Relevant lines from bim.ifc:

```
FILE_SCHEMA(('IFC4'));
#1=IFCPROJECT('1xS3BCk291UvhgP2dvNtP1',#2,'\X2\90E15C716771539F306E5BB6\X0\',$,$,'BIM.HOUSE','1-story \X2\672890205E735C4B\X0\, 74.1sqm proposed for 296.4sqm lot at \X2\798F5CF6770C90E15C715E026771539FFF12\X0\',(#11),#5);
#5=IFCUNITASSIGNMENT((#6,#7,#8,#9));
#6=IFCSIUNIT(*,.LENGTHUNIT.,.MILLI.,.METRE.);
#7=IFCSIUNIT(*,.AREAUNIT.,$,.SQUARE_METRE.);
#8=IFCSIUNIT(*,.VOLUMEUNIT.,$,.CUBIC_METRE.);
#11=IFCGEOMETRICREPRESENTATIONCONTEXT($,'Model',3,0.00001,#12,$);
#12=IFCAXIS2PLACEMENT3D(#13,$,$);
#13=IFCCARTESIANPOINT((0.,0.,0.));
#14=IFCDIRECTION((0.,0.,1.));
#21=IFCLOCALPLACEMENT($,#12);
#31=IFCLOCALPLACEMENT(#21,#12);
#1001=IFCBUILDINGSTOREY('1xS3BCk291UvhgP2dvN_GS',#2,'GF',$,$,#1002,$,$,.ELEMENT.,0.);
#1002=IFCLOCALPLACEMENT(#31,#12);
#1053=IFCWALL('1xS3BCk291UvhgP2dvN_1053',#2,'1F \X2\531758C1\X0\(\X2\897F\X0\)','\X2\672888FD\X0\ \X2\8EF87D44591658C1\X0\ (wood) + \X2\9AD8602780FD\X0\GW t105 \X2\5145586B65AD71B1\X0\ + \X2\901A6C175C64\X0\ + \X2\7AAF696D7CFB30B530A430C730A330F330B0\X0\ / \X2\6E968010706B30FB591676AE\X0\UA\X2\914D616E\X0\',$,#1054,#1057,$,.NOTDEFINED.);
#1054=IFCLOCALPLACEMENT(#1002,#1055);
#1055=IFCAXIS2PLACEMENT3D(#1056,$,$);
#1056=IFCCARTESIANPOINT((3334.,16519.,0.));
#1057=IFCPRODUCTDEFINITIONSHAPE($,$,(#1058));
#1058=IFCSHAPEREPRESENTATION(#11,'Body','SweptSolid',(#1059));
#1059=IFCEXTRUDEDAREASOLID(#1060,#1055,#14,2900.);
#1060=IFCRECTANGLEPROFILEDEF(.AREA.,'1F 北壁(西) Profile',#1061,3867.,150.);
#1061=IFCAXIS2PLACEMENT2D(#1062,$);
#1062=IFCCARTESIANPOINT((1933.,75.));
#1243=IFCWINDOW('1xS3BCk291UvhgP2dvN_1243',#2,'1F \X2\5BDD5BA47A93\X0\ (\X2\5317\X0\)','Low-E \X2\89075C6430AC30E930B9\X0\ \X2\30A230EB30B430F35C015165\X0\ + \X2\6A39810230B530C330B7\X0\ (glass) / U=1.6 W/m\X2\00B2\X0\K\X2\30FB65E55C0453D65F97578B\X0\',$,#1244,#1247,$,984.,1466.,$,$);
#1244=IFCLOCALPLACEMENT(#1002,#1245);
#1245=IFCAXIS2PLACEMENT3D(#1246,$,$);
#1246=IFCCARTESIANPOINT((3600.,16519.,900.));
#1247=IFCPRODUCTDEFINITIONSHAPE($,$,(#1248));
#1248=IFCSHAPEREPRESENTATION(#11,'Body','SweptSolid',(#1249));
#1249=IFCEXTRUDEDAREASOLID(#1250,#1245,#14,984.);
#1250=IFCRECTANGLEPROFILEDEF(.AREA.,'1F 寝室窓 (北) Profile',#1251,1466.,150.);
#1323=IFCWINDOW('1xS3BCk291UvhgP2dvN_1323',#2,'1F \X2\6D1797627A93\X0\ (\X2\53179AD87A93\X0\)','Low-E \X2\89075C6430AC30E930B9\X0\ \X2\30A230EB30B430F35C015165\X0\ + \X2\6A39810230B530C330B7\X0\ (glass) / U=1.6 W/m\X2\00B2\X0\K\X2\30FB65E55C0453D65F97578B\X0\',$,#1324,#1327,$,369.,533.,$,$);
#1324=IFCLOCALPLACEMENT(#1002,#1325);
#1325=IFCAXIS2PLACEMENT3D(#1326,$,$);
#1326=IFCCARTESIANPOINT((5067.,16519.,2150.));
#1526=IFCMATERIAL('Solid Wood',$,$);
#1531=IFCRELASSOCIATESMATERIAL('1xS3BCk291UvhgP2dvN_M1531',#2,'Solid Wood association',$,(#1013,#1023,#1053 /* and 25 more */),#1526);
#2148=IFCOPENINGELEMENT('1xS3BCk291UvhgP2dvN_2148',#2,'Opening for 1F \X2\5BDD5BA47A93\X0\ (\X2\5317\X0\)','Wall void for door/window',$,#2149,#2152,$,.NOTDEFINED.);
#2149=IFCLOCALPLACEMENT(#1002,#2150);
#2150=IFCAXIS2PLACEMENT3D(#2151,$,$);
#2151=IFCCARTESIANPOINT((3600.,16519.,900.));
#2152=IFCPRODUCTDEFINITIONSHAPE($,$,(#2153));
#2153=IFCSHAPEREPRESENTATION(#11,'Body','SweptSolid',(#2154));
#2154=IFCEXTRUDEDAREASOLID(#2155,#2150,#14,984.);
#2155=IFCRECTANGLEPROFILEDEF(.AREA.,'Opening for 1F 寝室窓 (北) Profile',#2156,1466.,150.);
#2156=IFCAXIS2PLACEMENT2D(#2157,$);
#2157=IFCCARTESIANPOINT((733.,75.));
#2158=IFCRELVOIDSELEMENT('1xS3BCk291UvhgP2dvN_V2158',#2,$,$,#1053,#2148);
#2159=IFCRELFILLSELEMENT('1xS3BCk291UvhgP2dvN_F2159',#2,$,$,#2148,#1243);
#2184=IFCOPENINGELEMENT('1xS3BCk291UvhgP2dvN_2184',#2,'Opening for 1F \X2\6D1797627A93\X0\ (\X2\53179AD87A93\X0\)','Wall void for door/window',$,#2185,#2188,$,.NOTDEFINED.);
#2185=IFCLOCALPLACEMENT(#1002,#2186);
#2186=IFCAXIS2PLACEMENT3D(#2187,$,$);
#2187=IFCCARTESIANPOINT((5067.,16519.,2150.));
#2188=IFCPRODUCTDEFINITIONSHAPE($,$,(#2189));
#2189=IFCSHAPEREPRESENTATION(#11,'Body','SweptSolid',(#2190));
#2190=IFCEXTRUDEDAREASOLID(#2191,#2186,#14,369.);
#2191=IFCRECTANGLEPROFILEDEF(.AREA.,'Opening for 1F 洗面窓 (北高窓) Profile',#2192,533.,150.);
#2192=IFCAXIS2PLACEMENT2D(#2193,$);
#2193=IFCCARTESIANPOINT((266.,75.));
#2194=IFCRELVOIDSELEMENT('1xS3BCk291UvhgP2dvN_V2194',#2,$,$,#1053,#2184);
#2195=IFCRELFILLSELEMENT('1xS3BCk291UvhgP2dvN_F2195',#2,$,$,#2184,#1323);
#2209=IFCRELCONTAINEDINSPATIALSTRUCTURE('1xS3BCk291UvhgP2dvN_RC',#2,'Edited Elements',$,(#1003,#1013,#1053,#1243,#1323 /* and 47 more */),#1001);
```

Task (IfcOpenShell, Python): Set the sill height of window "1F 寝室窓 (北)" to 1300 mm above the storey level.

```python
import numpy as np
import ifcopenshell
import ifcopenshell.api.geometry
import ifcopenshell.geom
import ifcopenshell.util.element
import ifcopenshell.util.placement
import ifcopenshell.util.shape
import ifcopenshell.util.unit

model = ifcopenshell.open("bim.ifc")
unit_scale = ifcopenshell.util.unit.calculate_unit_scale(model)

window = model.by_id(1243)
opening = window.FillsVoids[0].RelatingOpeningElement
storey = ifcopenshell.util.element.get_container(window, ifc_class="IfcBuildingStorey")
level = ifcopenshell.util.placement.get_local_placement(storey.ObjectPlacement)[2, 3]

# The opening's origin need not be at the sill, so measure its lowest point.
shape = ifcopenshell.geom.create_shape(ifcopenshell.geom.settings(), opening)
bottom = ifcopenshell.util.shape.get_shape_bottom_elevation(shape, shape.geometry) / unit_scale
dz = level + 1.3 / unit_scale - bottom

shift = np.array([0.0, 0.0, dz])
# The window is not placed relative to its opening, so move both.
for product in (opening, window):
    matrix = ifcopenshell.util.placement.get_local_placement(product.ObjectPlacement)
    matrix[:3, 3] += shift
    ifcopenshell.api.geometry.edit_object_placement(model, product=product, matrix=matrix, is_si=False)

print(f"moved by {dz * unit_scale:+.3f} m")

model.write("bim_updated.ifc")
```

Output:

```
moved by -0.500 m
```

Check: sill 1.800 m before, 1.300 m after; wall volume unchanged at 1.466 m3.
